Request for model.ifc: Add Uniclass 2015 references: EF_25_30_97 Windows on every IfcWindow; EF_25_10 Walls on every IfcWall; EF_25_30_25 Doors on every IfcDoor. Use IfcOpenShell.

First a look at what the model holds.

```python
import ifcopenshell

model = ifcopenshell.open("model.ifc")
print(model.schema)
print("classifications:", [c.Name for c in model.by_type("IfcClassification")])
for ifc_class in ("IfcDoor", "IfcRoof", "IfcStair", "IfcWall", "IfcWindow"):
    print(ifc_class, len(model.by_type(ifc_class)))
```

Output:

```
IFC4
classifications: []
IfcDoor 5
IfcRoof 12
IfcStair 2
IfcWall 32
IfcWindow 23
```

```python
import ifcopenshell
import ifcopenshell.api.classification

model = ifcopenshell.open("model.ifc")

system = ifcopenshell.api.classification.add_classification(model, classification="Uniclass 2015")

codes = {
    "IfcWindow": ("EF_25_30_97", "Windows"),
    "IfcWall": ("EF_25_10", "Walls"),
    "IfcDoor": ("EF_25_30_25", "Doors"),
}
for ifc_class, (code, name) in codes.items():
    products = model.by_type(ifc_class)
    ifcopenshell.api.classification.add_reference(
        model, products=products, classification=system, identification=code, name=name
    )
    print(code, len(products))

model.write("model_v2.ifc")
```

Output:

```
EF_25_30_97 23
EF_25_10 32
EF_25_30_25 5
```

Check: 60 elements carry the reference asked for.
